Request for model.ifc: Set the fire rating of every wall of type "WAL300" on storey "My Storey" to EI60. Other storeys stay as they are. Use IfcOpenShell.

First a look at what the model holds.

```python
import ifcopenshell
import ifcopenshell.util.element

model = ifcopenshell.open("model.ifc")
print(model.schema)
storey = next(s for s in model.by_type("IfcBuildingStorey") if s.Name == "My Storey")
walls = [e for e in ifcopenshell.util.element.get_decomposition(storey) if e.is_a("IfcWall")]
seen = {}
for e in walls:
    element_type = ifcopenshell.util.element.get_type(e)
    key = (element_type.Name if element_type != e and element_type else None, ifcopenshell.util.element.get_pset(e, "Pset_WallCommon", "FireRating"))
    seen[key] = seen.get(key, 0) + 1
for (name, value), count in sorted(seen.items(), key=str):
    print(count, "x", name, "|", value)
```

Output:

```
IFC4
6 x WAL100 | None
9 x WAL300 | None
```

```python
import ifcopenshell
import ifcopenshell.api.pset
import ifcopenshell.util.element

model = ifcopenshell.open("model.ifc")

storey = next(s for s in model.by_type("IfcBuildingStorey") if s.Name == "My Storey")
walls = [e for e in ifcopenshell.util.element.get_decomposition(storey) if e.is_a("IfcWall")]

count = 0
for e in walls:
    element_type = ifcopenshell.util.element.get_type(e)
    if element_type in (None, e) or element_type.Name != "WAL300":
        continue
    # add_pset returns the element's existing set when there is one.
    pset = ifcopenshell.api.pset.add_pset(model, product=e, name="Pset_WallCommon")
    ifcopenshell.api.pset.edit_pset(model, pset=pset, properties={"FireRating": "EI60"})
    count += 1

print(count, "walls updated")

model.write("model_v2.ifc")
```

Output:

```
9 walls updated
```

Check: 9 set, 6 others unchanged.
